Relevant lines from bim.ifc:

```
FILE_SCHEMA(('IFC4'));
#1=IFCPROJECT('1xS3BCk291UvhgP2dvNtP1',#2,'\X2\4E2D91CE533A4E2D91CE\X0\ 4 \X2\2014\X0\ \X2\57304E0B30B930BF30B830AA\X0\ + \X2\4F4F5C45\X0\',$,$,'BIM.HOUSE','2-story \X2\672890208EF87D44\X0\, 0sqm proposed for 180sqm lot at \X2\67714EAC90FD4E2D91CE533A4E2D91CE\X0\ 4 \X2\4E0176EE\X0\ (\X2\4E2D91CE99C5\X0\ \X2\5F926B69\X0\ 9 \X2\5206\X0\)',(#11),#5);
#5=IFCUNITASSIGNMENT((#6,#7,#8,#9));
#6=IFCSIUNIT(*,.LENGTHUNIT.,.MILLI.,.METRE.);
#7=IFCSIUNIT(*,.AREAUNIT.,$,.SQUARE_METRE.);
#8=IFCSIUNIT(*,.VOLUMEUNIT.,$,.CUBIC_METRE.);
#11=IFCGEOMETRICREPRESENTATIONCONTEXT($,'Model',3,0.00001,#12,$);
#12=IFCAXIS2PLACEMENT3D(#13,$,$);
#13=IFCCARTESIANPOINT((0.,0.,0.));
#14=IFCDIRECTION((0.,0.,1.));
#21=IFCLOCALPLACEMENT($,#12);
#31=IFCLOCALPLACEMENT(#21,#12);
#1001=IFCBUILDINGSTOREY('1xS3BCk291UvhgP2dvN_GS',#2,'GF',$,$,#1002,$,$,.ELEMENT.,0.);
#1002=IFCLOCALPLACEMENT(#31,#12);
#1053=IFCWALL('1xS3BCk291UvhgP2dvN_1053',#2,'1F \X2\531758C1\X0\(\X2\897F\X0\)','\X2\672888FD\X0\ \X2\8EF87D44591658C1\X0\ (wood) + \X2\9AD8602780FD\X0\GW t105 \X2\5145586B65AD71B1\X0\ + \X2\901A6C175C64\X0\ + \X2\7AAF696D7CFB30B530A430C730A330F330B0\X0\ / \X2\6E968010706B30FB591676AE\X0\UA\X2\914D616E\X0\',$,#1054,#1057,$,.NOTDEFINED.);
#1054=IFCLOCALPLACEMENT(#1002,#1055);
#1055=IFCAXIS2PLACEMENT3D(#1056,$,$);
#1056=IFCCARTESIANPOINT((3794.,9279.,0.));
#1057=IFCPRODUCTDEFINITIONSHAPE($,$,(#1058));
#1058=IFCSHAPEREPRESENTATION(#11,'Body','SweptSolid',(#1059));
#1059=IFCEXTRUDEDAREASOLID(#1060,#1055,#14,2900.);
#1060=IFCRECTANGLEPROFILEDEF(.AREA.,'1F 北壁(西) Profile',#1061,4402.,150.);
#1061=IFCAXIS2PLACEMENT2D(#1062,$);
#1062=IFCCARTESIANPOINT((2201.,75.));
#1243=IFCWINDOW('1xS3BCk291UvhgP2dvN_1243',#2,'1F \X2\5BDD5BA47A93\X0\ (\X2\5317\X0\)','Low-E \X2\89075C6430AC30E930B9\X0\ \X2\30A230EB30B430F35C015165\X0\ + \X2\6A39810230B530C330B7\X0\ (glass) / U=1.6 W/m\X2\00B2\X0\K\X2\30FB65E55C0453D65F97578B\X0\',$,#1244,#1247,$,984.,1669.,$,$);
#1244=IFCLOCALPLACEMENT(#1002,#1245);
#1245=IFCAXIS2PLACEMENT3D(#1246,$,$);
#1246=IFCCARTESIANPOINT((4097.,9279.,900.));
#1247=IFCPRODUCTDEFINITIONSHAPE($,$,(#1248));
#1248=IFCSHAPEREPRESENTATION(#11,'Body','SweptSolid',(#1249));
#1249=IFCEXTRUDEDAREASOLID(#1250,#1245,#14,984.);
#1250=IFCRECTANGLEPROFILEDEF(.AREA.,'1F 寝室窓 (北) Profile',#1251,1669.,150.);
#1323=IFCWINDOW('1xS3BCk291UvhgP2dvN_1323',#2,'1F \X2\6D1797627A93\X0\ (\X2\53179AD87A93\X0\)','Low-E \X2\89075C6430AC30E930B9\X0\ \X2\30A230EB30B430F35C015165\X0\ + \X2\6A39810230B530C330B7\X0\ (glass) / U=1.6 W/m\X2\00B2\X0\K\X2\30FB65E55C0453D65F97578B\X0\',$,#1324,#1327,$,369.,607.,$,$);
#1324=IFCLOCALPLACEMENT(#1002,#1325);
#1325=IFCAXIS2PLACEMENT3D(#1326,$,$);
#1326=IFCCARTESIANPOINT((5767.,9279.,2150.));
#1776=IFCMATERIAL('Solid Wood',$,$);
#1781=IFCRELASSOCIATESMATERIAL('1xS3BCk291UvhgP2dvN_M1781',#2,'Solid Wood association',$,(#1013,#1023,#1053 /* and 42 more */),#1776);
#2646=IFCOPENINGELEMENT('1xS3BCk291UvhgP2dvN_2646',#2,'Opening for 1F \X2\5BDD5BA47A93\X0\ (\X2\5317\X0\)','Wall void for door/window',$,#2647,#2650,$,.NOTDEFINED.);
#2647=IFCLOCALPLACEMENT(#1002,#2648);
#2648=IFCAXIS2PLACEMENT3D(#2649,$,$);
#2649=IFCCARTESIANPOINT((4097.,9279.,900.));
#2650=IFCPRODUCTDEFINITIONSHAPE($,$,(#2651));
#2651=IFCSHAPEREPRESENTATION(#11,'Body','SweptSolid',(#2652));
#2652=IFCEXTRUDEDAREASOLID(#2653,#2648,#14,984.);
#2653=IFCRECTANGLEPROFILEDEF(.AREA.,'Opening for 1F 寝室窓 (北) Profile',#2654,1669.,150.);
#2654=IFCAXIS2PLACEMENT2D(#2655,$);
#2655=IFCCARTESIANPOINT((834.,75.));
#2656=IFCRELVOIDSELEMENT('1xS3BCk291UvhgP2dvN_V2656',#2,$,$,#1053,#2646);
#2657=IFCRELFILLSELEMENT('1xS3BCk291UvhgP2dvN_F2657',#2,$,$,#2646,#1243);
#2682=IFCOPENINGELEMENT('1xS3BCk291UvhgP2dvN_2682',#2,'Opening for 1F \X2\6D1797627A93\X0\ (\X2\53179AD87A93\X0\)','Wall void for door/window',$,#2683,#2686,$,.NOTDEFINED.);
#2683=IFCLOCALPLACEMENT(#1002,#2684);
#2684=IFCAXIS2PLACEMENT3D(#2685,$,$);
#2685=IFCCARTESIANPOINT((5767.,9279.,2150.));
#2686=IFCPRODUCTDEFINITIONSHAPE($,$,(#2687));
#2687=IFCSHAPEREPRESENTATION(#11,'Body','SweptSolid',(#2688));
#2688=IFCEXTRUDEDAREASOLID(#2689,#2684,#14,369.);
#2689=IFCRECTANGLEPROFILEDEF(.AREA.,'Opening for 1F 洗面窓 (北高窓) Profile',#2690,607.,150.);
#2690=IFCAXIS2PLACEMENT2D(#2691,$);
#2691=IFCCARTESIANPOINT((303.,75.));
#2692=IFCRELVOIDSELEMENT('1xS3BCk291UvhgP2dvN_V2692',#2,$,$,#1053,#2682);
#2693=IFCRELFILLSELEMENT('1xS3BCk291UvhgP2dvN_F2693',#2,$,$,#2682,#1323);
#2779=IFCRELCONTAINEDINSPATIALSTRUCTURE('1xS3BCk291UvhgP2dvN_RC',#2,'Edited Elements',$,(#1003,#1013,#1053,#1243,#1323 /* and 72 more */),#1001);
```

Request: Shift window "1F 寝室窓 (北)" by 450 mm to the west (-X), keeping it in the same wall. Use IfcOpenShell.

```python
import ifcopenshell
import ifcopenshell.api.geometry
import ifcopenshell.util.placement

model = ifcopenshell.open("bim.ifc")

window = model.by_guid("1xS3BCk291UvhgP2dvN_1243")
opening = window.FillsVoids[0].RelatingOpeningElement
wall = opening.VoidsElements[0].RelatingBuildingElement

wall_matrix = ifcopenshell.util.placement.get_local_placement(wall.ObjectPlacement)
shift = wall_matrix[:3, 0] * -450.0
before = ifcopenshell.util.placement.get_local_placement(window.ObjectPlacement)[:3, 3].copy()

# The window is not placed relative to its opening, so move both.
for product in (opening, window):
    matrix = ifcopenshell.util.placement.get_local_placement(product.ObjectPlacement)
    matrix[:3, 3] += shift
    ifcopenshell.api.geometry.edit_object_placement(model, product=product, matrix=matrix, is_si=False)

after = ifcopenshell.util.placement.get_local_placement(window.ObjectPlacement)[:3, 3]
print("window moved by", (after - before).round(3) + 0.0)

model.write("bim-out.ifc")
```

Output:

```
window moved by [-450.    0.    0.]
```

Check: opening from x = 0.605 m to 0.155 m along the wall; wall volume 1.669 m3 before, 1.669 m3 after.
